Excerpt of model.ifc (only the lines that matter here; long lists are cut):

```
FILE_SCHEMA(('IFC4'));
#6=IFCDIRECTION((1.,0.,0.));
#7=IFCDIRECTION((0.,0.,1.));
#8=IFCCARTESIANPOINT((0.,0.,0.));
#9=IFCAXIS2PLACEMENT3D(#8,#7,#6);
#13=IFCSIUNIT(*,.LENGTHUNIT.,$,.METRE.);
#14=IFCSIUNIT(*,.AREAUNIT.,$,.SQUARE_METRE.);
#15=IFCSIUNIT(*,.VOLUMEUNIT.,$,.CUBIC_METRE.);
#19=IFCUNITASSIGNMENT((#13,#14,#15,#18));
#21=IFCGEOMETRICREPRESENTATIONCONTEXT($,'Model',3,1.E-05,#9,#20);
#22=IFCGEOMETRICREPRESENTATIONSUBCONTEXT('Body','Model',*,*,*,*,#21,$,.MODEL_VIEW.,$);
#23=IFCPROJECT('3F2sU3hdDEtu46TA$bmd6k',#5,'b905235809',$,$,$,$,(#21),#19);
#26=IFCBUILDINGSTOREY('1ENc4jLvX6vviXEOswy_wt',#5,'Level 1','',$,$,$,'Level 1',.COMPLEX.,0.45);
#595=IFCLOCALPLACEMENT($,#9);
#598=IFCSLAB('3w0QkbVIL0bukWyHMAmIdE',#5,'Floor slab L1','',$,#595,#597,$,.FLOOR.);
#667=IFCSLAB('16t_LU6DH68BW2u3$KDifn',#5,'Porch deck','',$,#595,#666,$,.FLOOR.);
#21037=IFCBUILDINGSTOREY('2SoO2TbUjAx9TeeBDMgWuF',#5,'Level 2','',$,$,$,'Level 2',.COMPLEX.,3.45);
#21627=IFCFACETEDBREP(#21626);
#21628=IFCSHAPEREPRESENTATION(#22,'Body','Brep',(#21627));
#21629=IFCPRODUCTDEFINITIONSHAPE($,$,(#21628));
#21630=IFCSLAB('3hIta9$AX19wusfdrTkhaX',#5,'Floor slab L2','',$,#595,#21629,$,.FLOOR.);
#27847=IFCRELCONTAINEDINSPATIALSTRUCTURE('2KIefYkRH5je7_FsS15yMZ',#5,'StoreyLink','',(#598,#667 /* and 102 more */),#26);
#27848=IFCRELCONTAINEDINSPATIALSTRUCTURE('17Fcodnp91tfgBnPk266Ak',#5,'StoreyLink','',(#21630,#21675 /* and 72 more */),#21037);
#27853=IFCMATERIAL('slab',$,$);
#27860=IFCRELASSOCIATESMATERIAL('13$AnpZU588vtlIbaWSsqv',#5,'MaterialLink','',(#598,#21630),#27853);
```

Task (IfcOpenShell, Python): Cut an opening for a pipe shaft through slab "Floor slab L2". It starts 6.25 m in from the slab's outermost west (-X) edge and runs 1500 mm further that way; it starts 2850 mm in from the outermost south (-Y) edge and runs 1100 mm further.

```python
import numpy as np
import ifcopenshell
import ifcopenshell.api.feature
import ifcopenshell.api.geometry
import ifcopenshell.api.root
import ifcopenshell.geom
import ifcopenshell.util.placement
import ifcopenshell.util.representation
import ifcopenshell.util.shape
import ifcopenshell.util.unit

model = ifcopenshell.open("model.ifc")
unit_scale = ifcopenshell.util.unit.calculate_unit_scale(model)
settings = ifcopenshell.geom.settings()


def volume(element):
    """Net volume in cubic metres, openings subtracted."""
    shape = ifcopenshell.geom.create_shape(settings, element)
    return ifcopenshell.util.shape.get_volume(shape.geometry)


slab = model.by_guid("3hIta9$AX19wusfdrTkhaX")
before = volume(slab)

# Extent in the slab's own axes, in metres. The edges named are its -X and -Y sides.
slab_shape = ifcopenshell.geom.create_shape(settings, slab)
vertices = ifcopenshell.util.shape.get_vertices(slab_shape.geometry)
x_min, y_min, bottom = vertices.min(axis=0)
top = vertices[:, 2].max()

opening = ifcopenshell.api.root.create_entity(model, ifc_class="IfcOpeningElement", name="Pipe shaft opening", predefined_type="OPENING")
context = ifcopenshell.util.representation.get_context(model, "Model", "Body", "MODEL_VIEW")
width, depth = 1.5, 1.1
outline = [(0.0, 0.0), (width, 0.0), (width, depth), (0.0, depth), (0.0, 0.0)]
# Overshoot both faces by 50 mm so the cut is clean.
shape = ifcopenshell.api.geometry.add_slab_representation(
    model, context=context, depth=top - bottom + 0.1, polyline=outline
)
ifcopenshell.api.geometry.assign_representation(model, product=opening, representation=shape)

matrix = ifcopenshell.util.placement.get_local_placement(slab.ObjectPlacement)
matrix[:, 3] = matrix @ np.append(np.array([x_min + 6.25, y_min + 2.85, bottom - 0.05]) / unit_scale, 1.0)
ifcopenshell.api.geometry.edit_object_placement(model, product=opening, matrix=matrix, is_si=False)
ifcopenshell.api.feature.add_feature(model, feature=opening, element=slab)

after = volume(slab)

print(f"slab volume {before:.3f} -> {after:.3f} m3")

model.write("model_edited.ifc")
```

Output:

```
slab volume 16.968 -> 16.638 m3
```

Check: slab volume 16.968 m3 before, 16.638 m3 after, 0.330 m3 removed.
